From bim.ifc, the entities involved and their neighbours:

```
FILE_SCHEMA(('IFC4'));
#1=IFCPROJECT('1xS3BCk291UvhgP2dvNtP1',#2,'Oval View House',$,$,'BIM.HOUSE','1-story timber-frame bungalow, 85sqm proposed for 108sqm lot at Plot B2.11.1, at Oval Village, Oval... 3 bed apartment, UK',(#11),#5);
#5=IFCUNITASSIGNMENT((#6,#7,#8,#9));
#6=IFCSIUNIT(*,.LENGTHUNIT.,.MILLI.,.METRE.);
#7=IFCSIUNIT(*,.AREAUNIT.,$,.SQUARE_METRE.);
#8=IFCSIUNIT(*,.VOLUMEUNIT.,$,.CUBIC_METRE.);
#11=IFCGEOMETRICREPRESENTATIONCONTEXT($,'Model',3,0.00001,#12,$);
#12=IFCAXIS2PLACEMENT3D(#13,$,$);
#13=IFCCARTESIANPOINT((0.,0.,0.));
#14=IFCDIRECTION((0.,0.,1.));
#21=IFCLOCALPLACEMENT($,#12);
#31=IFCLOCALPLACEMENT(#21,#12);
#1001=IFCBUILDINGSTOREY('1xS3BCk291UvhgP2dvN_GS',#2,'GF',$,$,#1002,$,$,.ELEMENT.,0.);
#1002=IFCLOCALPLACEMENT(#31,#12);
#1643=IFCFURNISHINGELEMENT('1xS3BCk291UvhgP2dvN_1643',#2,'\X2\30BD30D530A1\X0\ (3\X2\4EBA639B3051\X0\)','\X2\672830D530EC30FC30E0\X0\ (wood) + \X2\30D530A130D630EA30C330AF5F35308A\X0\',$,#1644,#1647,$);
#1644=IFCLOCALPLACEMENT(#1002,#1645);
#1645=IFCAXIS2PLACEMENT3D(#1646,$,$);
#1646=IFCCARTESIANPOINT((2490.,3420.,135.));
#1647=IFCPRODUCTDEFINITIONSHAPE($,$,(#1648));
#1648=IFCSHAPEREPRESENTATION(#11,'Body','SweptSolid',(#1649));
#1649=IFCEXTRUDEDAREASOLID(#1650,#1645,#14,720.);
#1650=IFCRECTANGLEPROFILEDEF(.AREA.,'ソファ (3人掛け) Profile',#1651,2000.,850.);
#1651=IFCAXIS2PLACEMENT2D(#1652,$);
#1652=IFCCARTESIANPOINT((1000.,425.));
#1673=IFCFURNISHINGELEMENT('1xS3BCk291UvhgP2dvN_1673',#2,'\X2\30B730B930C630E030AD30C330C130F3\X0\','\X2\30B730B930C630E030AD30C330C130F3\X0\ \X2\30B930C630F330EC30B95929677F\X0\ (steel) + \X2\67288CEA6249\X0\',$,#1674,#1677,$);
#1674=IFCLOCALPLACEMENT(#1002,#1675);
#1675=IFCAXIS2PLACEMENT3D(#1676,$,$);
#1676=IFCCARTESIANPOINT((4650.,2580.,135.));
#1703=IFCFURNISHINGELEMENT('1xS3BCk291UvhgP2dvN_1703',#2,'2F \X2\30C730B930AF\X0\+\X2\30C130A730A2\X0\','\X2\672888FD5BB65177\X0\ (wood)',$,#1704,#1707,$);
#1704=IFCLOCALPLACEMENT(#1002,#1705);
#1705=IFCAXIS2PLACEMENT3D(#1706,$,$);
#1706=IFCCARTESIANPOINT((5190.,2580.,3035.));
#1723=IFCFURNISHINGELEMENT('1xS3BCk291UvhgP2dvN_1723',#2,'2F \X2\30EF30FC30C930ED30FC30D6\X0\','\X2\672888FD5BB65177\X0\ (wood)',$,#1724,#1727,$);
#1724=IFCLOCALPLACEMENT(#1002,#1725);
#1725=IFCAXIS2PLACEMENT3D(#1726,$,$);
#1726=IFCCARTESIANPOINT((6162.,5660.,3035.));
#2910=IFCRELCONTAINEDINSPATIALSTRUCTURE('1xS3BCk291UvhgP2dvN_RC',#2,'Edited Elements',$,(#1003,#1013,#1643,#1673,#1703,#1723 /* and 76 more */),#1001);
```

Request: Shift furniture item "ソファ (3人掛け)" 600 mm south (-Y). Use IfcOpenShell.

```python
import ifcopenshell
import ifcopenshell.api.geometry
import ifcopenshell.util.placement

model = ifcopenshell.open("bim.ifc")

item = model.by_guid("1xS3BCk291UvhgP2dvN_1643")
matrix = ifcopenshell.util.placement.get_local_placement(item.ObjectPlacement)
matrix[1, 3] -= 600.0
ifcopenshell.api.geometry.edit_object_placement(model, product=item, matrix=matrix, is_si=False)

print(ifcopenshell.util.placement.get_local_placement(item.ObjectPlacement).round(3) + 0.0)

model.write("bim-out.ifc")
```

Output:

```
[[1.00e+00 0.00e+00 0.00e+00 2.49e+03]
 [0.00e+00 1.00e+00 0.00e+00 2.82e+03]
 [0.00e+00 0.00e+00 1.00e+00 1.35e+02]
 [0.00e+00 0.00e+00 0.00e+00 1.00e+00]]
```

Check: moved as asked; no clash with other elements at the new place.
